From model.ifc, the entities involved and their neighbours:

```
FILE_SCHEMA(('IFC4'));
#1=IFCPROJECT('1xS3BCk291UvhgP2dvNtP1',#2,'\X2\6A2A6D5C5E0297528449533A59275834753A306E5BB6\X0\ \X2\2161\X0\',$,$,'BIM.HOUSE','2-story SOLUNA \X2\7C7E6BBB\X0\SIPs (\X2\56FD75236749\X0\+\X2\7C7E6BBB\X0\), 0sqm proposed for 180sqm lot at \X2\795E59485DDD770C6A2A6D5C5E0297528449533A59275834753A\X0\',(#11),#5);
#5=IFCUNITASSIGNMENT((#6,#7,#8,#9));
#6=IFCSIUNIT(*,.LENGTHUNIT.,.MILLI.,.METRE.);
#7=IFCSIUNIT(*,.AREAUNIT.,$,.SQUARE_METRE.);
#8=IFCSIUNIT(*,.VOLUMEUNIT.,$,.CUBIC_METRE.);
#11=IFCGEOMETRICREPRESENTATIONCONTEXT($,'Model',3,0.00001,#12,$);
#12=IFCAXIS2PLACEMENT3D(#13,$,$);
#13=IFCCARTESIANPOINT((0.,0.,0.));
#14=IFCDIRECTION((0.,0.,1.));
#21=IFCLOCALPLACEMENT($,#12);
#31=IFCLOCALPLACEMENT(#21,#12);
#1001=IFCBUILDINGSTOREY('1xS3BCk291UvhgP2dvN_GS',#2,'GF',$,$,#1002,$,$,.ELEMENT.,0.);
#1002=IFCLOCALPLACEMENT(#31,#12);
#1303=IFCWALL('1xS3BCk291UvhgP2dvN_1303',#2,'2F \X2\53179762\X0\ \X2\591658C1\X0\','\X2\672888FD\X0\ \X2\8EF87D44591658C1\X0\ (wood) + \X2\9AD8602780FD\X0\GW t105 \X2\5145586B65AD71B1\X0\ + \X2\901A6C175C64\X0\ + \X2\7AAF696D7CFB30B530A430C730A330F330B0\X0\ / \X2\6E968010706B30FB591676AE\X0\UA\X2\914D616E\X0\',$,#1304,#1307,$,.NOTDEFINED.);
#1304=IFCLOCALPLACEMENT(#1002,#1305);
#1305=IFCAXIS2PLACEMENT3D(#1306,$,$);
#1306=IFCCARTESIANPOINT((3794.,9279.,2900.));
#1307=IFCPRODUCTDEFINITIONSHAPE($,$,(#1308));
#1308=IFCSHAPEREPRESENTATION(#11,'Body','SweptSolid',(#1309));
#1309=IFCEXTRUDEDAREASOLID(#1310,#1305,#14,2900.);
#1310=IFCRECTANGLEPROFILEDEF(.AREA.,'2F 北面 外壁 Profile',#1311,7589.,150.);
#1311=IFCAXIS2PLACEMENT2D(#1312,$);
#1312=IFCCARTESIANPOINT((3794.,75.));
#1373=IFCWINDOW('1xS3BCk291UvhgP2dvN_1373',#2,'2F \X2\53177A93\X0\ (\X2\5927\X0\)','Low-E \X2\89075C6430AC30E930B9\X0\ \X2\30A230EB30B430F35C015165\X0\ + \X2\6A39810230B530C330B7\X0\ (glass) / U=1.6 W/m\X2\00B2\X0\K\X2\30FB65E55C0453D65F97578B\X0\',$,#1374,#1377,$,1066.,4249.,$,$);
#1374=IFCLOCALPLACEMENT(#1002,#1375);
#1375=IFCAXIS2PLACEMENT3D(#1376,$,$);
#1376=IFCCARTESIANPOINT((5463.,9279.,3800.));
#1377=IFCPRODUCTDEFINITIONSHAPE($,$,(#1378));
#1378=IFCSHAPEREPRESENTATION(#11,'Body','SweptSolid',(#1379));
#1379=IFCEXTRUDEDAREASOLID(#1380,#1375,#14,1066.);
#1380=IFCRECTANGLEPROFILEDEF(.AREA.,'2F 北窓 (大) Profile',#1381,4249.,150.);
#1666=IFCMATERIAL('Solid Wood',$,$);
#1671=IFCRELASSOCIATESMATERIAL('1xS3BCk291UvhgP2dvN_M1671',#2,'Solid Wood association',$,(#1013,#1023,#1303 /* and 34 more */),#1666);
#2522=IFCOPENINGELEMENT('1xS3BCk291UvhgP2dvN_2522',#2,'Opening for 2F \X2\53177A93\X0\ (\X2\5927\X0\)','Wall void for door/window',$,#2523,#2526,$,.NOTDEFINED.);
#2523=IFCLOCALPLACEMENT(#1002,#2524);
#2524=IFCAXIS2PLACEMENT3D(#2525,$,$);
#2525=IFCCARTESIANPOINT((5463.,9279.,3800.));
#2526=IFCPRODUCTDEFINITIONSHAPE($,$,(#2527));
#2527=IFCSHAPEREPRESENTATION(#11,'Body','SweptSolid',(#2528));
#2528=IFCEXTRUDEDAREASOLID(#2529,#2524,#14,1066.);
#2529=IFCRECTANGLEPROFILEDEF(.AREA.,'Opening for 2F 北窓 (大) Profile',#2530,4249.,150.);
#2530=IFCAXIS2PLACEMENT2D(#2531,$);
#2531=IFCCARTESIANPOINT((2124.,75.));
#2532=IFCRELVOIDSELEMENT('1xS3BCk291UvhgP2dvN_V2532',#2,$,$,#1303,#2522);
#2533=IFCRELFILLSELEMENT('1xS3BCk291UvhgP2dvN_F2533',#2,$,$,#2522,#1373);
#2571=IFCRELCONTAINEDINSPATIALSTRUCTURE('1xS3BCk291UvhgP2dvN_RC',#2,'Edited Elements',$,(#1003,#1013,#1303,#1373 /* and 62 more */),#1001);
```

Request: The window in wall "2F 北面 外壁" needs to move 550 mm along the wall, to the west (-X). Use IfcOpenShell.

```python
import ifcopenshell
import ifcopenshell.api.geometry
import ifcopenshell.util.placement
import ifcopenshell.util.unit

model = ifcopenshell.open("model.ifc")
unit_scale = ifcopenshell.util.unit.calculate_unit_scale(model)

window = model.by_guid("1xS3BCk291UvhgP2dvN_1373")
opening = window.FillsVoids[0].RelatingOpeningElement
wall = opening.VoidsElements[0].RelatingBuildingElement

wall_matrix = ifcopenshell.util.placement.get_local_placement(wall.ObjectPlacement)
shift = wall_matrix[:3, 0] * -0.55 / unit_scale
before = ifcopenshell.util.placement.get_local_placement(window.ObjectPlacement)[:3, 3].copy()

# The window is not placed relative to its opening, so move both.
for product in (opening, window):
    matrix = ifcopenshell.util.placement.get_local_placement(product.ObjectPlacement)
    matrix[:3, 3] += shift
    ifcopenshell.api.geometry.edit_object_placement(model, product=product, matrix=matrix, is_si=False)

after = ifcopenshell.util.placement.get_local_placement(window.ObjectPlacement)[:3, 3]
print("window moved by", (after - before).round(3) + 0.0)

model.write("model-out.ifc")
```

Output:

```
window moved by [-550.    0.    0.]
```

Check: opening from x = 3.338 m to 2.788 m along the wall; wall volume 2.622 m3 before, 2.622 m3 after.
